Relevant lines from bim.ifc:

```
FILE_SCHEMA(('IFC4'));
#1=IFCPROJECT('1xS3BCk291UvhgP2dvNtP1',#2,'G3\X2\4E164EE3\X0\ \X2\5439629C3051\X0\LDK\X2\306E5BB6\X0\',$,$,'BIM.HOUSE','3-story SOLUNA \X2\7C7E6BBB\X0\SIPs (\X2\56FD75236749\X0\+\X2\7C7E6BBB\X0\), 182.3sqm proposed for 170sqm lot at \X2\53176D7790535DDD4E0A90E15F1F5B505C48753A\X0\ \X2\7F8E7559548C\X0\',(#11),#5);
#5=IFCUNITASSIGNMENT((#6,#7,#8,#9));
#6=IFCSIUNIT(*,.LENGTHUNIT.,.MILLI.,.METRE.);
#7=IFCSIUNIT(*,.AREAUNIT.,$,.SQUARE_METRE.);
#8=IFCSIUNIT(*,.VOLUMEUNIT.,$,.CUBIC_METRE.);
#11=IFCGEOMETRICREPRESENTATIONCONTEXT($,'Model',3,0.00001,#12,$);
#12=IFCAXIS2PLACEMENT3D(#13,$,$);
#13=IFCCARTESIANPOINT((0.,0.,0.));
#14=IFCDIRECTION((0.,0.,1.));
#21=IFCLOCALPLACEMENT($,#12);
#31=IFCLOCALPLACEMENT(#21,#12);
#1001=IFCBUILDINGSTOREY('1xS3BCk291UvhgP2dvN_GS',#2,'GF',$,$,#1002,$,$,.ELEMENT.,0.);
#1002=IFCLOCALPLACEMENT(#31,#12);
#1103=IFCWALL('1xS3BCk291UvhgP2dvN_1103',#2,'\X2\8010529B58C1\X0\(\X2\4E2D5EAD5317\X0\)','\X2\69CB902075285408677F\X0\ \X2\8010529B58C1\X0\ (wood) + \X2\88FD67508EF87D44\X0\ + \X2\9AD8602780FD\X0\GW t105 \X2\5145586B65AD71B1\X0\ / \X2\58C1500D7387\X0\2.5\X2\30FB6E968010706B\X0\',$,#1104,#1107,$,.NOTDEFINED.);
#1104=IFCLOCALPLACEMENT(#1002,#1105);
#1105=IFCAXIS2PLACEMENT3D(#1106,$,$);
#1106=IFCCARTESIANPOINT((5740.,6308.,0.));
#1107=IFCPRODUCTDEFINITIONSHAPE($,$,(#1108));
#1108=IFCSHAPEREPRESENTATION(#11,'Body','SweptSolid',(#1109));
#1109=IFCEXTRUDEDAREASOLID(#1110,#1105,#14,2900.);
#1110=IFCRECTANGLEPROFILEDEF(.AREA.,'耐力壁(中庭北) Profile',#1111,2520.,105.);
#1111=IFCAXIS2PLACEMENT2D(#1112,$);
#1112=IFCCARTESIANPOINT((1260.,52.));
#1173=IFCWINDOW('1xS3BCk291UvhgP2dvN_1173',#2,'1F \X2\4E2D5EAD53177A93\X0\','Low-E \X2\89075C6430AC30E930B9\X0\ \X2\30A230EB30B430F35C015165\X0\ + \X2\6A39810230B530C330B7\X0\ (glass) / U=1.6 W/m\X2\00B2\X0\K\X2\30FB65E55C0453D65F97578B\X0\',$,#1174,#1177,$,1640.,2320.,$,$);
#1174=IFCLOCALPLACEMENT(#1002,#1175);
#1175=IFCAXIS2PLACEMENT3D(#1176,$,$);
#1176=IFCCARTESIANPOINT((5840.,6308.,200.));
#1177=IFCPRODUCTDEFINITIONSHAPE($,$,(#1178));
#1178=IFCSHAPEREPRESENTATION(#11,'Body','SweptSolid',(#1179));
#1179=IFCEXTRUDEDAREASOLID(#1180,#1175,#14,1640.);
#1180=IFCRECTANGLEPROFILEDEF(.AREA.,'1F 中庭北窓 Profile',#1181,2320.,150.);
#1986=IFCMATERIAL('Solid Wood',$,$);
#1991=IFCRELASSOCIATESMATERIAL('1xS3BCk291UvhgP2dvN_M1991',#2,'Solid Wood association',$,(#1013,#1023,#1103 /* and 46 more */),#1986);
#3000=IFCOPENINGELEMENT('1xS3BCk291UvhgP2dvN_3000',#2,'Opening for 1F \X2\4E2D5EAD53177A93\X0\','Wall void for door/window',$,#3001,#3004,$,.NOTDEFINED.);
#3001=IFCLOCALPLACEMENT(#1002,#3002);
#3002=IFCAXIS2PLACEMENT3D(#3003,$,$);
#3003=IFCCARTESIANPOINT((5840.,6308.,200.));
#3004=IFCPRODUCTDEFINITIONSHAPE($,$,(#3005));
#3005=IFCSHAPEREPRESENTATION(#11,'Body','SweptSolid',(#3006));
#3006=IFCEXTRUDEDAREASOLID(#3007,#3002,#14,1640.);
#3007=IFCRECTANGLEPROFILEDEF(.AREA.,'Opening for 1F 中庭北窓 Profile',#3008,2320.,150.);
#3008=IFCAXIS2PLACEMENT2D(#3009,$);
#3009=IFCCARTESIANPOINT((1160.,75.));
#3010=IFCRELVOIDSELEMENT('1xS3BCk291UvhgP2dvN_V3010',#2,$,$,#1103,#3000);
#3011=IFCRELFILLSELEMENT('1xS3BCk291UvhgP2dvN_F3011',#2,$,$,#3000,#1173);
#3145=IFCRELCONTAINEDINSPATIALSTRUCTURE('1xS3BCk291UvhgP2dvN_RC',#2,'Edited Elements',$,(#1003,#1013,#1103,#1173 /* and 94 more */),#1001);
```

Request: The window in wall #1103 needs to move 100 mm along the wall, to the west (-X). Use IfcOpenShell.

```python
import ifcopenshell
import ifcopenshell.api.geometry
import ifcopenshell.util.placement

model = ifcopenshell.open("bim.ifc")

window = model.by_guid("1xS3BCk291UvhgP2dvN_1173")
opening = window.FillsVoids[0].RelatingOpeningElement
wall = opening.VoidsElements[0].RelatingBuildingElement

wall_matrix = ifcopenshell.util.placement.get_local_placement(wall.ObjectPlacement)
shift = wall_matrix[:3, 0] * -100.0
before = ifcopenshell.util.placement.get_local_placement(window.ObjectPlacement)[:3, 3].copy()

# The window is not placed relative to its opening, so move both.
for product in (opening, window):
    matrix = ifcopenshell.util.placement.get_local_placement(product.ObjectPlacement)
    matrix[:3, 3] += shift
    ifcopenshell.api.geometry.edit_object_placement(model, product=product, matrix=matrix, is_si=False)

after = ifcopenshell.util.placement.get_local_placement(window.ObjectPlacement)[:3, 3]
print("window moved by", (after - before).round(3) + 0.0)

model.write("bim-out.ifc")
```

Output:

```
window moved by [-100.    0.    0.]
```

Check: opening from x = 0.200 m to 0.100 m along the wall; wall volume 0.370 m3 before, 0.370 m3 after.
